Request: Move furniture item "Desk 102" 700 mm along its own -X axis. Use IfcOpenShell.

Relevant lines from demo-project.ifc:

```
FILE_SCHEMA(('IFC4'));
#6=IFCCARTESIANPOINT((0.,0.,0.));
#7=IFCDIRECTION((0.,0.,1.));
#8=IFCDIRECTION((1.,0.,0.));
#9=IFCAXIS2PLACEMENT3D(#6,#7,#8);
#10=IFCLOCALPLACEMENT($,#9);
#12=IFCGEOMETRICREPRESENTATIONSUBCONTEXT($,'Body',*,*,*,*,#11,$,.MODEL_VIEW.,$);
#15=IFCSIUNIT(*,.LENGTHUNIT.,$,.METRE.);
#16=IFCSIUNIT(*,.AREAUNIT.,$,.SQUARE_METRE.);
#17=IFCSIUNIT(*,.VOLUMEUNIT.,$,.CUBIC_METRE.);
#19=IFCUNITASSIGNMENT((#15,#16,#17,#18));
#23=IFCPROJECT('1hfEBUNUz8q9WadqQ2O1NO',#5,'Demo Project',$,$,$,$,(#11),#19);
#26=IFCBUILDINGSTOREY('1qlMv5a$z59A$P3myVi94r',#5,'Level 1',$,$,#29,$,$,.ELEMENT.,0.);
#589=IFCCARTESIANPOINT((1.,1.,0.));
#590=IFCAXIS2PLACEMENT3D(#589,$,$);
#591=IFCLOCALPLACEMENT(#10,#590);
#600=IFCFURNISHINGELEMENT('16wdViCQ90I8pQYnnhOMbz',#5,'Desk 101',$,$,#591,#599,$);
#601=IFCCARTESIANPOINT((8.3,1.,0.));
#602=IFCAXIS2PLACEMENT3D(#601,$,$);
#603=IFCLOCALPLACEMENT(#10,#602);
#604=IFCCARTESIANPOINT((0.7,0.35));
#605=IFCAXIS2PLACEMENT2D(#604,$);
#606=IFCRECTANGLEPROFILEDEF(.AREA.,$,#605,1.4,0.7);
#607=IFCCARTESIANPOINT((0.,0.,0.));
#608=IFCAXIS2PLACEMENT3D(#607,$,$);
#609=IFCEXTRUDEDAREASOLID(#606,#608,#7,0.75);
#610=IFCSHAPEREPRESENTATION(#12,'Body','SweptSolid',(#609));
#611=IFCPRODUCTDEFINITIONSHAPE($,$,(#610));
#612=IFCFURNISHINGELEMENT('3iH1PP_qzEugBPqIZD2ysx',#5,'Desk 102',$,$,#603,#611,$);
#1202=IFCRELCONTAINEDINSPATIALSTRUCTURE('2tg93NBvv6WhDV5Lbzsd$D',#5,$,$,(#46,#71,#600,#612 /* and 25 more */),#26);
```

```python
import ifcopenshell
import ifcopenshell.api.geometry
import ifcopenshell.util.placement
import ifcopenshell.util.unit

model = ifcopenshell.open("demo-project.ifc")
unit_scale = ifcopenshell.util.unit.calculate_unit_scale(model)

item = model.by_id(612)
matrix = ifcopenshell.util.placement.get_local_placement(item.ObjectPlacement)
matrix[:3, 3] -= matrix[:3, 0] * 0.7 / unit_scale
ifcopenshell.api.geometry.edit_object_placement(model, product=item, matrix=matrix, is_si=False)

print(ifcopenshell.util.placement.get_local_placement(item.ObjectPlacement).round(3) + 0.0)

model.write("demo-project_rev.ifc")
```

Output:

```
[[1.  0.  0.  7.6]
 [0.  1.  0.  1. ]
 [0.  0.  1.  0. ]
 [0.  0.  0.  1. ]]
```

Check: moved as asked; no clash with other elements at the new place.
